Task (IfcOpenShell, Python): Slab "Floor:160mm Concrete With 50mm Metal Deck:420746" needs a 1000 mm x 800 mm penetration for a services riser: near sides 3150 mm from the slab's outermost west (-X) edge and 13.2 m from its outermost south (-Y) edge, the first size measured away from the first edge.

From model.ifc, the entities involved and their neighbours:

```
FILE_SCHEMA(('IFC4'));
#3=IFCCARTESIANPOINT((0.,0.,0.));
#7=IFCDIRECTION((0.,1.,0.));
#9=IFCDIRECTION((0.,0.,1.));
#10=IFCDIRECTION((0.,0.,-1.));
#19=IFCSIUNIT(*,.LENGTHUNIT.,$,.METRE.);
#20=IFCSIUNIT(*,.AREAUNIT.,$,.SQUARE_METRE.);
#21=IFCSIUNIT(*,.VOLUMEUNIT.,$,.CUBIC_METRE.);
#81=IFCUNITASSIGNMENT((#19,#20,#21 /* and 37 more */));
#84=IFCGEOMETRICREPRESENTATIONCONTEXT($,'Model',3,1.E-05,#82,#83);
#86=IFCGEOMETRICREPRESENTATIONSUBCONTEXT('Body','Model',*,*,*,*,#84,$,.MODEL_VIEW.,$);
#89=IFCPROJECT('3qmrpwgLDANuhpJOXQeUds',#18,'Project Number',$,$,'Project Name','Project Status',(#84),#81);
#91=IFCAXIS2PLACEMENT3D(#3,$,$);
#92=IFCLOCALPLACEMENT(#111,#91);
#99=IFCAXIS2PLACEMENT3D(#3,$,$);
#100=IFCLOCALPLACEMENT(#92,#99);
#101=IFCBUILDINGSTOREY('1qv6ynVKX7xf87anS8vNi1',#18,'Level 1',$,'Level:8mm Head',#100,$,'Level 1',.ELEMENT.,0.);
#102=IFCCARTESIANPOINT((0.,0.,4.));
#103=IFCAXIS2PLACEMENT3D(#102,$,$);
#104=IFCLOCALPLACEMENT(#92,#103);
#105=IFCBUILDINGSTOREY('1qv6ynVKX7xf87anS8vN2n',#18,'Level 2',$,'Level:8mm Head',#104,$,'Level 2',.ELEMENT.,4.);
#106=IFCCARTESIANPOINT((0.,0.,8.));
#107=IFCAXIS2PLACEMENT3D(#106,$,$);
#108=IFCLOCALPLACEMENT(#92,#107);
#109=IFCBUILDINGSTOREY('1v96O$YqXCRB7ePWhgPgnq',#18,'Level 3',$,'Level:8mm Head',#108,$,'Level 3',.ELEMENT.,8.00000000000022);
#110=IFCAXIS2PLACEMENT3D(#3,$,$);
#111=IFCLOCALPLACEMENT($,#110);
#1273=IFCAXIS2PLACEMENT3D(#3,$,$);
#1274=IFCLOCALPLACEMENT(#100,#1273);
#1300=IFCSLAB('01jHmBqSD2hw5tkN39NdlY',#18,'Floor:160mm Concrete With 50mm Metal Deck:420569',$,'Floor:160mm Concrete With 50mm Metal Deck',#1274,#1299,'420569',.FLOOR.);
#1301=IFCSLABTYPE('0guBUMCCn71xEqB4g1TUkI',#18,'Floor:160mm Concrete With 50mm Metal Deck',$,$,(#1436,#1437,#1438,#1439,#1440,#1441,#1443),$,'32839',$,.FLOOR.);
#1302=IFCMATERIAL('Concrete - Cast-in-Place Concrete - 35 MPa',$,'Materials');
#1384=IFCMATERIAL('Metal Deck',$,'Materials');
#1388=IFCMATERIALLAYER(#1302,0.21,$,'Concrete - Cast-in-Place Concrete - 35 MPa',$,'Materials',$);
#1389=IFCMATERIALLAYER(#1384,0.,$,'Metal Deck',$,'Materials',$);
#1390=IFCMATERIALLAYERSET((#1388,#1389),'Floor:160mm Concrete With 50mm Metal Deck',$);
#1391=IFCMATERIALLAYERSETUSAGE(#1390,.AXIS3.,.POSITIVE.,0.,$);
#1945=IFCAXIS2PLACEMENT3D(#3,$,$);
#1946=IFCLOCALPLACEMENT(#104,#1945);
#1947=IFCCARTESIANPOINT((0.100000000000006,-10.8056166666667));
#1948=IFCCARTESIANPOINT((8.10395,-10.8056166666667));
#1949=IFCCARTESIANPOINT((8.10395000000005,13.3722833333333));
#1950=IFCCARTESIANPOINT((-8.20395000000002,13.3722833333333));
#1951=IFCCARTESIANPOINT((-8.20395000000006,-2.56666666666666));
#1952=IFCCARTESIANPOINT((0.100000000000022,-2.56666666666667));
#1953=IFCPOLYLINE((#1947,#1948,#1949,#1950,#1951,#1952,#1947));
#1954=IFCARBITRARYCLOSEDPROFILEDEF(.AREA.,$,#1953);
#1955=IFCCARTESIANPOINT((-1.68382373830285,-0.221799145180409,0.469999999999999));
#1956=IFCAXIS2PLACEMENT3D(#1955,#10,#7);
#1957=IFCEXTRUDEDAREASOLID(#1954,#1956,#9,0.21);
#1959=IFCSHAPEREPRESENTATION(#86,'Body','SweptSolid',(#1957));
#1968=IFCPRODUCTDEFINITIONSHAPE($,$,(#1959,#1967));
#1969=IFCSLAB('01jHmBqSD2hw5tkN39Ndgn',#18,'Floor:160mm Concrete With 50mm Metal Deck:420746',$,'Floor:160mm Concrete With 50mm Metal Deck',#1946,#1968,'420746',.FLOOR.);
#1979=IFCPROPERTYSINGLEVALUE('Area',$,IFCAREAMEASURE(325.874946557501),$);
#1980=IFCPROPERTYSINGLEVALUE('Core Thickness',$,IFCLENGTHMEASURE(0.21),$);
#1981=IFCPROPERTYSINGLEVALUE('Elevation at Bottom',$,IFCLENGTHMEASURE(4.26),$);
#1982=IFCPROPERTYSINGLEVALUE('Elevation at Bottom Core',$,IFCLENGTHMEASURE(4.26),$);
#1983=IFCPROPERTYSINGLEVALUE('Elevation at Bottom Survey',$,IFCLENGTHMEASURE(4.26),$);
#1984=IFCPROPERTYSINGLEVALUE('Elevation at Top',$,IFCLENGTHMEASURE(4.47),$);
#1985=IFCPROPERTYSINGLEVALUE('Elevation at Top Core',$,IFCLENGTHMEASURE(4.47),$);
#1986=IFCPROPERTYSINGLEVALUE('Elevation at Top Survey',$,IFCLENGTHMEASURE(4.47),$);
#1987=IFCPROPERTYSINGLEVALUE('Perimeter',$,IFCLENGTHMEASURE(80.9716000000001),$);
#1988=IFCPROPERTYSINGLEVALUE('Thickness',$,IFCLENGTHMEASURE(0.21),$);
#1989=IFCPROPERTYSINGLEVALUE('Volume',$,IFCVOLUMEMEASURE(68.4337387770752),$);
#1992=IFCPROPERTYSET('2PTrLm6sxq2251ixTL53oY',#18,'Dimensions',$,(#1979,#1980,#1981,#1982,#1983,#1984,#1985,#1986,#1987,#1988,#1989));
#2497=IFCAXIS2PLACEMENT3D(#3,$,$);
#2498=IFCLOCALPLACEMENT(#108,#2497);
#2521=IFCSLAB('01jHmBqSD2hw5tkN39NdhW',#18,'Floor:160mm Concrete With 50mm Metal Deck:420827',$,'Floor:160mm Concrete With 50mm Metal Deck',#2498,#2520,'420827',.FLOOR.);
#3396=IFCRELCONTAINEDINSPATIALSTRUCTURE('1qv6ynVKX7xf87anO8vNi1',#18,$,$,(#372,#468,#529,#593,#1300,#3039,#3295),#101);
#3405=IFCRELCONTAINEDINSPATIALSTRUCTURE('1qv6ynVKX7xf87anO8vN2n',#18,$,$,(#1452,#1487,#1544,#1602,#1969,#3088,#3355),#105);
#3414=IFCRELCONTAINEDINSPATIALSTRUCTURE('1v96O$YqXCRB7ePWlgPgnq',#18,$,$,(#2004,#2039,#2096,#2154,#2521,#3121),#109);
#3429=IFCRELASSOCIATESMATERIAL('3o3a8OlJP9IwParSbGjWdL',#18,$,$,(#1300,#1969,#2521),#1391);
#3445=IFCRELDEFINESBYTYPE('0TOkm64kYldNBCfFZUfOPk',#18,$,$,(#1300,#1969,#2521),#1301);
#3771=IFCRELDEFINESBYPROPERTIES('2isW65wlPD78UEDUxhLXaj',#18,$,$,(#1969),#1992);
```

```python
import numpy as np
import ifcopenshell
import ifcopenshell.api.feature
import ifcopenshell.api.geometry
import ifcopenshell.api.pset
import ifcopenshell.api.root
import ifcopenshell.geom
import ifcopenshell.util.element
import ifcopenshell.util.placement
import ifcopenshell.util.representation
import ifcopenshell.util.shape
import ifcopenshell.util.unit

model = ifcopenshell.open("model.ifc")
unit_scale = ifcopenshell.util.unit.calculate_unit_scale(model)
area_scale = ifcopenshell.util.unit.calculate_unit_scale(model, "AREAUNIT")
volume_scale = ifcopenshell.util.unit.calculate_unit_scale(model, "VOLUMEUNIT")
settings = ifcopenshell.geom.settings()


def volume(element):
    """Net volume in cubic metres, openings subtracted."""
    shape = ifcopenshell.geom.create_shape(settings, element)
    return ifcopenshell.util.shape.get_volume(shape.geometry)


slab = model.by_id(1969)
before = volume(slab)

# Extent in the slab's own axes, in metres. The edges named are its -X and -Y sides.
slab_shape = ifcopenshell.geom.create_shape(settings, slab)
vertices = ifcopenshell.util.shape.get_vertices(slab_shape.geometry)
x_min, y_min, bottom = vertices.min(axis=0)
top = vertices[:, 2].max()

opening = ifcopenshell.api.root.create_entity(model, ifc_class="IfcOpeningElement", name="Services riser opening", predefined_type="OPENING")
context = ifcopenshell.util.representation.get_context(model, "Model", "Body", "MODEL_VIEW")
width, depth = 1, 0.8
outline = [(0.0, 0.0), (width, 0.0), (width, depth), (0.0, depth), (0.0, 0.0)]
# Overshoot both faces by 50 mm so the cut is clean.
shape = ifcopenshell.api.geometry.add_slab_representation(
    model, context=context, depth=top - bottom + 0.1, polyline=outline
)
ifcopenshell.api.geometry.assign_representation(model, product=opening, representation=shape)

matrix = ifcopenshell.util.placement.get_local_placement(slab.ObjectPlacement)
matrix[:, 3] = matrix @ np.append(np.array([x_min + 3.15, y_min + 13.2, bottom - 0.05]) / unit_scale, 1.0)
ifcopenshell.api.geometry.edit_object_placement(model, product=opening, matrix=matrix, is_si=False)
ifcopenshell.api.feature.add_feature(model, feature=opening, element=slab)

after = volume(slab)

# Update the slab's stored quantities.
pset = model.by_id(ifcopenshell.util.element.get_pset(slab, "Dimensions", should_inherit=False)["id"])
ifcopenshell.api.pset.edit_pset(model, pset=pset, properties={
    "Area": model.create_entity("IfcAreaMeasure", after / (top - bottom) / area_scale),
    "Volume": model.create_entity("IfcVolumeMeasure", after / volume_scale),
})

print(f"slab volume {before:.3f} -> {after:.3f} m3")

model.write("model-out.ifc")
```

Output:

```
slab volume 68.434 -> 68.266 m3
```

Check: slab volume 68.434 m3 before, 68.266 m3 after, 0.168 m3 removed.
